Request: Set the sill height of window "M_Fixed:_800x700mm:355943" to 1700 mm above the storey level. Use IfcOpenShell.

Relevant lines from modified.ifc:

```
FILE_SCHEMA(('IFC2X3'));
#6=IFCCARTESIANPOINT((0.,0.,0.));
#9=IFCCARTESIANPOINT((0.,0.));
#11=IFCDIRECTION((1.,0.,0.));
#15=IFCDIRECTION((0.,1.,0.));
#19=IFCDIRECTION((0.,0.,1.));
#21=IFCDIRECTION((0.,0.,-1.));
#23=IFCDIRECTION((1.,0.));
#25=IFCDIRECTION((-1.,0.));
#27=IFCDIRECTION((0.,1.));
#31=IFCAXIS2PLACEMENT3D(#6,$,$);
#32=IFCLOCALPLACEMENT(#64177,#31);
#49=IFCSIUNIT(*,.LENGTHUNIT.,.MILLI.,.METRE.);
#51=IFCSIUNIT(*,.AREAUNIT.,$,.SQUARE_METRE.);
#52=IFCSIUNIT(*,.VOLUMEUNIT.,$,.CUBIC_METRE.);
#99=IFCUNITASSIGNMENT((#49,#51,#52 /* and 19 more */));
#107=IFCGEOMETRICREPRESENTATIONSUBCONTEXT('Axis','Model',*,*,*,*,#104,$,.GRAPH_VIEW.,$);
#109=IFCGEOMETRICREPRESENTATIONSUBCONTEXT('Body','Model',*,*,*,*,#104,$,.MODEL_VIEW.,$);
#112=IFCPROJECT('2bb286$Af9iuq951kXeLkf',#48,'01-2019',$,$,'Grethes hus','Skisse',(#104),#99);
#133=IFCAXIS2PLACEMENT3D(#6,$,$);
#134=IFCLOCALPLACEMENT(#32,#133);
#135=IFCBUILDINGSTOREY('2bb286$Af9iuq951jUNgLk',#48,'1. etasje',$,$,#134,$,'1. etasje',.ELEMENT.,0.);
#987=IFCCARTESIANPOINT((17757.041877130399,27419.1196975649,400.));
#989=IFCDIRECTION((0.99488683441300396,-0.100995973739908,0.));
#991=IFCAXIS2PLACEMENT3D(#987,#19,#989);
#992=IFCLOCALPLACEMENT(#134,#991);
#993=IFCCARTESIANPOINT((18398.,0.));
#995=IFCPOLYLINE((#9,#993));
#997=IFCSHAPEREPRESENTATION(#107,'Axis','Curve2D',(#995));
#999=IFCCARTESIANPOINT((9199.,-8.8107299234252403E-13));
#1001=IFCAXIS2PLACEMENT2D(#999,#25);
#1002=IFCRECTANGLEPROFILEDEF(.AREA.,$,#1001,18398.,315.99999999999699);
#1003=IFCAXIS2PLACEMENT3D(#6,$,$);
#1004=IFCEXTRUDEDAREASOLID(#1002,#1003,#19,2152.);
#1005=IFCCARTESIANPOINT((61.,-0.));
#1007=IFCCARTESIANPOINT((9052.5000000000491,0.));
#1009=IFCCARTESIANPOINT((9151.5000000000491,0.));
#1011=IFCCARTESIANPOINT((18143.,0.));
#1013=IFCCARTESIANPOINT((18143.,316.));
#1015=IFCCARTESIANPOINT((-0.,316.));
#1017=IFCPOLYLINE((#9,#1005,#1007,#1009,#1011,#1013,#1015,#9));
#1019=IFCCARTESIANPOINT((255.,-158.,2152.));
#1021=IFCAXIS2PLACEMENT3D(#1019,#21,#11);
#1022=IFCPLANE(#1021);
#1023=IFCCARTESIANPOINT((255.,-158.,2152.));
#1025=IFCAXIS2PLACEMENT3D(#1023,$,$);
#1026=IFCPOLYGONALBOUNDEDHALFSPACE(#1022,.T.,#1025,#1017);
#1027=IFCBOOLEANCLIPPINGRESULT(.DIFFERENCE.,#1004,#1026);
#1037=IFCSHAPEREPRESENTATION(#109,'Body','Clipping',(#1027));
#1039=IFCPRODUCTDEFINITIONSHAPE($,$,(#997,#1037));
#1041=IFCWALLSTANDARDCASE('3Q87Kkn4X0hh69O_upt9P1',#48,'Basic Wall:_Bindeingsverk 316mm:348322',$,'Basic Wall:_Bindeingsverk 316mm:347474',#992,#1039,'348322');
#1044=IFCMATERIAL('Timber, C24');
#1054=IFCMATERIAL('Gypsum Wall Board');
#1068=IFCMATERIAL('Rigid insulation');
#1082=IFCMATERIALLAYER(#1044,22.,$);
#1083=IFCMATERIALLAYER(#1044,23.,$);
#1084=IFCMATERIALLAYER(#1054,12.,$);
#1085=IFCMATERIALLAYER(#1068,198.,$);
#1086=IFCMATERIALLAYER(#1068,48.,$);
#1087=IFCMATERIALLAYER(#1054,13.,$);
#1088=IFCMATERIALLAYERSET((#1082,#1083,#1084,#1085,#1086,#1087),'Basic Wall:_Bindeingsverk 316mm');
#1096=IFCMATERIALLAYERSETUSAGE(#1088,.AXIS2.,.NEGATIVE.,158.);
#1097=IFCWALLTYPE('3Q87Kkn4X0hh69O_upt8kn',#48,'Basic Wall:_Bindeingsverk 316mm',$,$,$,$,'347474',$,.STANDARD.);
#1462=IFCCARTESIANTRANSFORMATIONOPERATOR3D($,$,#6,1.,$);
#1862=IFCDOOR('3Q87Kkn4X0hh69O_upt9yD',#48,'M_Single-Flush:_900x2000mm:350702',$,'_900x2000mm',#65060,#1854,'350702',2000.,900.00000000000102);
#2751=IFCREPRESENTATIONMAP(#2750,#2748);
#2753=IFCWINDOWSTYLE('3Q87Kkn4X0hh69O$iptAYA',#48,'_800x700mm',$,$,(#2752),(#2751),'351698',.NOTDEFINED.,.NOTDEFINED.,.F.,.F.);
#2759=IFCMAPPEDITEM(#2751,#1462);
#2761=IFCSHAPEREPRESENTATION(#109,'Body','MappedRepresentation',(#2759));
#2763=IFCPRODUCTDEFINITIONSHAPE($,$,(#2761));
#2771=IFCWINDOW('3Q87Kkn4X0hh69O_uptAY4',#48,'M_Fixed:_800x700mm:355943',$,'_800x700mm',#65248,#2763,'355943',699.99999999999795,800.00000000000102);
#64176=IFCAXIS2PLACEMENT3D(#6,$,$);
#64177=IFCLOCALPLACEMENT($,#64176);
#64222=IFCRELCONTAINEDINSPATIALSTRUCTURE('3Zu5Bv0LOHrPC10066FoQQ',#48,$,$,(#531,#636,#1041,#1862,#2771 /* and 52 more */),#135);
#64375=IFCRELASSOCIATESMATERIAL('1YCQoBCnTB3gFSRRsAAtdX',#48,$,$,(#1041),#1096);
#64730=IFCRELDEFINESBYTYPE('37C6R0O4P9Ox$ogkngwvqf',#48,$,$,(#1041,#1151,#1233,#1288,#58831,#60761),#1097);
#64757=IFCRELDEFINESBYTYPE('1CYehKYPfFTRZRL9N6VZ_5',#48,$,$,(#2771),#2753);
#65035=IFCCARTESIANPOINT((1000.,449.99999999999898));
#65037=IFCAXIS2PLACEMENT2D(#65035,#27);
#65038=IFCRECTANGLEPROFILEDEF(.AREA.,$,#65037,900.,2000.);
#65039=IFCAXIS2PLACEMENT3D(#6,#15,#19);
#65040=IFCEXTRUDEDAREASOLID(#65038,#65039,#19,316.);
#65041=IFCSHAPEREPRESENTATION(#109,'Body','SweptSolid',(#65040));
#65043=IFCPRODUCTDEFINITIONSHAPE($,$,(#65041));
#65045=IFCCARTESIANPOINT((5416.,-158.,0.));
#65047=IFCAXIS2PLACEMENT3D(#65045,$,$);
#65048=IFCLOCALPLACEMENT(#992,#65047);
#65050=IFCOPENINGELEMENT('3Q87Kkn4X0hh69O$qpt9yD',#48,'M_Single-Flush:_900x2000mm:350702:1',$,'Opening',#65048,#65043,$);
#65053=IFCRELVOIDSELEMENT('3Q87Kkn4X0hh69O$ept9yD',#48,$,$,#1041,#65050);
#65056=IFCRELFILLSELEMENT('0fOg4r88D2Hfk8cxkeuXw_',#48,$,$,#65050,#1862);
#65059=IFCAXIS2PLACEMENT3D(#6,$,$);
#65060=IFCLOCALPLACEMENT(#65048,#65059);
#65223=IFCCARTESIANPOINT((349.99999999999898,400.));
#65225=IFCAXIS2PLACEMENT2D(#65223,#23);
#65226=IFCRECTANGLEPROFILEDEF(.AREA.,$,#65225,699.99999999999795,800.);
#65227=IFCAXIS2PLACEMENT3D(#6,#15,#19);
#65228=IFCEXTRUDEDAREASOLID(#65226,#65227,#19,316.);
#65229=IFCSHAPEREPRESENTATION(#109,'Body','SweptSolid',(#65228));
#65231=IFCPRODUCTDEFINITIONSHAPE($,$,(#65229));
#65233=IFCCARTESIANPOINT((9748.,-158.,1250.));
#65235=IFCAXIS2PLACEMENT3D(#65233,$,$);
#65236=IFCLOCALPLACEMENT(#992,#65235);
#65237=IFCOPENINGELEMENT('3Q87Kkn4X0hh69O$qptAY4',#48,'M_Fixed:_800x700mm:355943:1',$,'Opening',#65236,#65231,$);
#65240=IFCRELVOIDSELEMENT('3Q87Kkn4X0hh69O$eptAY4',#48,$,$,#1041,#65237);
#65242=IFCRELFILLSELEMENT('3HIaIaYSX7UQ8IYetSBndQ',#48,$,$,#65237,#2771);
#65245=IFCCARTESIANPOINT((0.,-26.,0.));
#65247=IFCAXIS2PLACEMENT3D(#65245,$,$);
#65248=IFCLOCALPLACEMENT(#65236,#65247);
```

```python
import numpy as np
import ifcopenshell
import ifcopenshell.api.geometry
import ifcopenshell.geom
import ifcopenshell.util.element
import ifcopenshell.util.placement
import ifcopenshell.util.shape
import ifcopenshell.util.unit

model = ifcopenshell.open("modified.ifc")
unit_scale = ifcopenshell.util.unit.calculate_unit_scale(model)

window = model.by_guid("3Q87Kkn4X0hh69O_uptAY4")
opening = window.FillsVoids[0].RelatingOpeningElement
storey = ifcopenshell.util.element.get_container(window, ifc_class="IfcBuildingStorey")
level = ifcopenshell.util.placement.get_local_placement(storey.ObjectPlacement)[2, 3]

# The opening's origin need not be at the sill, so measure its lowest point.
shape = ifcopenshell.geom.create_shape(ifcopenshell.geom.settings(), opening)
bottom = ifcopenshell.util.shape.get_shape_bottom_elevation(shape, shape.geometry) / unit_scale
dz = level + 1700.0 - bottom

shift = np.array([0.0, 0.0, dz])
# The window is placed relative to its opening, so it follows when the opening moves.
matrix = ifcopenshell.util.placement.get_local_placement(opening.ObjectPlacement)
matrix[:3, 3] += shift
ifcopenshell.api.geometry.edit_object_placement(
    model, product=opening, matrix=matrix, is_si=False, should_transform_children=True
)

print(f"moved by {dz * unit_scale:+.3f} m")

model.write("modified_rev.ifc")
```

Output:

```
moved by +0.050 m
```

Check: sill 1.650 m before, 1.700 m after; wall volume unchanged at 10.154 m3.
